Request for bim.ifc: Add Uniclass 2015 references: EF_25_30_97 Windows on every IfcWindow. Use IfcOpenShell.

First a look at what the model holds.

```python
import ifcopenshell

model = ifcopenshell.open("bim.ifc")
print(model.schema)
print("classifications:", [c.Name for c in model.by_type("IfcClassification")])
for ifc_class in ("IfcDoor", "IfcRoof", "IfcStair", "IfcWall", "IfcWindow"):
    print(ifc_class, len(model.by_type(ifc_class)))
```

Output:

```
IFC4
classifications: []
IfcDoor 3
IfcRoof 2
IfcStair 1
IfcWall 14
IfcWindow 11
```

```python
import ifcopenshell
import ifcopenshell.api.classification

model = ifcopenshell.open("bim.ifc")

system = ifcopenshell.api.classification.add_classification(model, classification="Uniclass 2015")

codes = {
    "IfcWindow": ("EF_25_30_97", "Windows"),
}
for ifc_class, (code, name) in codes.items():
    products = model.by_type(ifc_class)
    ifcopenshell.api.classification.add_reference(
        model, products=products, classification=system, identification=code, name=name
    )
    print(code, len(products))

model.write("bim-out.ifc")
```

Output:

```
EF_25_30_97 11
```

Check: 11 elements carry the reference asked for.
